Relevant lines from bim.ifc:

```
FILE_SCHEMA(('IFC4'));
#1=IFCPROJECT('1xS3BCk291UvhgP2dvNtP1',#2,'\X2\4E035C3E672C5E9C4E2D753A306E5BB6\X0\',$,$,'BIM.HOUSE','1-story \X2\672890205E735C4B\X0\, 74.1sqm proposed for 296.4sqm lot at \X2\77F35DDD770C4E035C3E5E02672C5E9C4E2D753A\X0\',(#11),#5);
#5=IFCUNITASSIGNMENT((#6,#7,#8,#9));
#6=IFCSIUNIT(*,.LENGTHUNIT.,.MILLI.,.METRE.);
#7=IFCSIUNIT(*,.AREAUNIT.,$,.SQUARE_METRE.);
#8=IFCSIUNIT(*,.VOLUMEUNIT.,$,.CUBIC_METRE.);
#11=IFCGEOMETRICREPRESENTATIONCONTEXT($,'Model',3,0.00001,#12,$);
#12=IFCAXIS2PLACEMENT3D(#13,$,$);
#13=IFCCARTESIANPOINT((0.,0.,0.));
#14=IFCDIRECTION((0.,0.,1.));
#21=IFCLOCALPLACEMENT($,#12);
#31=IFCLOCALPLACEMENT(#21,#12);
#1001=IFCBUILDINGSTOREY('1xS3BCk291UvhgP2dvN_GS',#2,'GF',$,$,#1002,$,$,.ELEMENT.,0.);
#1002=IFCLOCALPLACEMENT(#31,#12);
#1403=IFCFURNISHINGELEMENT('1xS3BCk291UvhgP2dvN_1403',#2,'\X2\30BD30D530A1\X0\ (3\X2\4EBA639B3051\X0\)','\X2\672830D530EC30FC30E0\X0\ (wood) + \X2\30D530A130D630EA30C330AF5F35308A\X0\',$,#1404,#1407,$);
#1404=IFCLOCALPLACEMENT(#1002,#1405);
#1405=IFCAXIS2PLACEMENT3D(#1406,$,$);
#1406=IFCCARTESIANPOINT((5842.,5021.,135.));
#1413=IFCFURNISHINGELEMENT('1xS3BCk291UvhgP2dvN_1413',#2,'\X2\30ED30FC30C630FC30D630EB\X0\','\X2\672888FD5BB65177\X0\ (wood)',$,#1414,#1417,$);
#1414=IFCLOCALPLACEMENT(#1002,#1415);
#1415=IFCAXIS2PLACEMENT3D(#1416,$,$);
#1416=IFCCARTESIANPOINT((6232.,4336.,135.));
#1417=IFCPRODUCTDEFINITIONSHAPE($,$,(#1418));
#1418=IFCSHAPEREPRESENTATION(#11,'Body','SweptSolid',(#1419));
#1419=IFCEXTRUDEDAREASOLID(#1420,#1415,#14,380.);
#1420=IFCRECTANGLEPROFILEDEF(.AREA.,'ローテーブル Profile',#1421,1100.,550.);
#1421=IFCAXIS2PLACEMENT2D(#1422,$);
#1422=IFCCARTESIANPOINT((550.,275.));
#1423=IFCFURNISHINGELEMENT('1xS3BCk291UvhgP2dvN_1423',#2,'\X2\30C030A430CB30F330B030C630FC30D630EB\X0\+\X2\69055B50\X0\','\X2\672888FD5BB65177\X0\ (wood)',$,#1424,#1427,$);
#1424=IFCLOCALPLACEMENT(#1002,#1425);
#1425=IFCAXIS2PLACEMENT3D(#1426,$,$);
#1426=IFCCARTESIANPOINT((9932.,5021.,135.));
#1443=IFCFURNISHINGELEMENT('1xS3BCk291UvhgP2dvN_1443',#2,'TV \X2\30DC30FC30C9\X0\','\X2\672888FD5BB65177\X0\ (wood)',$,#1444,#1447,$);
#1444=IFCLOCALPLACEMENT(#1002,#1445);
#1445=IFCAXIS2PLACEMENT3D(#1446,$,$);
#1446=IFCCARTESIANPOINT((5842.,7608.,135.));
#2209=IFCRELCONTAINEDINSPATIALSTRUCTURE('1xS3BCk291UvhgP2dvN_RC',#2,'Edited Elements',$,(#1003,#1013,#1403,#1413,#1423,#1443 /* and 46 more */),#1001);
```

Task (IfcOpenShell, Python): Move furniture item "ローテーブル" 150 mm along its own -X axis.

```python
import ifcopenshell
import ifcopenshell.api.geometry
import ifcopenshell.util.placement

model = ifcopenshell.open("bim.ifc")

item = model.by_id(1413)
matrix = ifcopenshell.util.placement.get_local_placement(item.ObjectPlacement)
matrix[:3, 3] -= matrix[:3, 0] * 150.0
ifcopenshell.api.geometry.edit_object_placement(model, product=item, matrix=matrix, is_si=False)

print(ifcopenshell.util.placement.get_local_placement(item.ObjectPlacement).round(3) + 0.0)

model.write("bim-out.ifc")
```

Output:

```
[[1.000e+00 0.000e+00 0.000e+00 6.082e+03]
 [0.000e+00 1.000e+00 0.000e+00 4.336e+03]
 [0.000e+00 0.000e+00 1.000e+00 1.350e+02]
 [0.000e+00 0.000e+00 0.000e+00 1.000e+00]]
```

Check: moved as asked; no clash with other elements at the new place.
